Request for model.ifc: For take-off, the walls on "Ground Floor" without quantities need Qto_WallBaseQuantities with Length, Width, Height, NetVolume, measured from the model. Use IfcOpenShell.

First a look at what the model holds.

```python
import ifcopenshell
import ifcopenshell.util.element
import ifcopenshell.util.unit

model = ifcopenshell.open("model.ifc")
print(model.schema)
for unit_type in ("LENGTHUNIT", "AREAUNIT", "VOLUMEUNIT"):
    print(unit_type, ifcopenshell.util.unit.calculate_unit_scale(model, unit_type))
storey = next(s for s in model.by_type("IfcBuildingStorey") if s.Name == "Ground Floor")
walls = [e for e in ifcopenshell.util.element.get_decomposition(storey) if e.is_a("IfcWall")]
for e in sorted(walls, key=lambda e: e.id()):
    print(e.id(), e.is_a(), e.Name, list(ifcopenshell.util.element.get_psets(e, qtos_only=True)), sep=" | ")
```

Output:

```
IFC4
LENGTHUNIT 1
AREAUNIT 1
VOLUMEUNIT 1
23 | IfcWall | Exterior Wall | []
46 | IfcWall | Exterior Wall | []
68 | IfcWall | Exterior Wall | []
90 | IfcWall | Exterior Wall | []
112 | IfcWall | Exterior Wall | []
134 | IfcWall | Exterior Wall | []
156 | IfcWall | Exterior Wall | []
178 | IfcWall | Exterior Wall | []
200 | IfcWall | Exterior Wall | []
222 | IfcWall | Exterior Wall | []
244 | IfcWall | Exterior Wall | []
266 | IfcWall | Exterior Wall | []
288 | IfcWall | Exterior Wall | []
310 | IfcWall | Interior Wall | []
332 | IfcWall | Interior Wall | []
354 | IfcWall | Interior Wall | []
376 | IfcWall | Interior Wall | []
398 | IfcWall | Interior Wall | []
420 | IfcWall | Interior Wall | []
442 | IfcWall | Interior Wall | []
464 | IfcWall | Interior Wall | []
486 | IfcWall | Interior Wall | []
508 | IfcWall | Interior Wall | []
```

```python
import ifcopenshell
import ifcopenshell.api.pset
import ifcopenshell.geom
import ifcopenshell.util.element
import ifcopenshell.util.shape
import ifcopenshell.util.unit

model = ifcopenshell.open("model.ifc")
unit_scale = ifcopenshell.util.unit.calculate_unit_scale(model)
volume_scale = ifcopenshell.util.unit.calculate_unit_scale(model, "VOLUMEUNIT")
settings = ifcopenshell.geom.settings()

storey = next(s for s in model.by_type("IfcBuildingStorey") if s.Name == "Ground Floor")
walls = [e for e in ifcopenshell.util.element.get_decomposition(storey) if e.is_a("IfcWall")]

for e in sorted(walls, key=lambda e: e.id()):
    if ifcopenshell.util.element.get_psets(e, qtos_only=True, should_inherit=False):
        continue
    # Geometry comes back in metres, in the element's own axes.
    shape = ifcopenshell.geom.create_shape(settings, e)
    values = {
        "Length": ifcopenshell.util.shape.get_x(shape.geometry) / unit_scale,
        "Width": ifcopenshell.util.shape.get_y(shape.geometry) / unit_scale,
        "Height": ifcopenshell.util.shape.get_z(shape.geometry) / unit_scale,
        "NetVolume": ifcopenshell.util.shape.get_volume(shape.geometry) / volume_scale,
    }
    qto = ifcopenshell.api.pset.add_qto(model, product=e, name="Qto_WallBaseQuantities")
    ifcopenshell.api.pset.edit_qto(model, qto=qto, properties=values)
    print(e.id(), {k: round(v, 3) for k, v in values.items()})

model.write("model_v2.ifc")
```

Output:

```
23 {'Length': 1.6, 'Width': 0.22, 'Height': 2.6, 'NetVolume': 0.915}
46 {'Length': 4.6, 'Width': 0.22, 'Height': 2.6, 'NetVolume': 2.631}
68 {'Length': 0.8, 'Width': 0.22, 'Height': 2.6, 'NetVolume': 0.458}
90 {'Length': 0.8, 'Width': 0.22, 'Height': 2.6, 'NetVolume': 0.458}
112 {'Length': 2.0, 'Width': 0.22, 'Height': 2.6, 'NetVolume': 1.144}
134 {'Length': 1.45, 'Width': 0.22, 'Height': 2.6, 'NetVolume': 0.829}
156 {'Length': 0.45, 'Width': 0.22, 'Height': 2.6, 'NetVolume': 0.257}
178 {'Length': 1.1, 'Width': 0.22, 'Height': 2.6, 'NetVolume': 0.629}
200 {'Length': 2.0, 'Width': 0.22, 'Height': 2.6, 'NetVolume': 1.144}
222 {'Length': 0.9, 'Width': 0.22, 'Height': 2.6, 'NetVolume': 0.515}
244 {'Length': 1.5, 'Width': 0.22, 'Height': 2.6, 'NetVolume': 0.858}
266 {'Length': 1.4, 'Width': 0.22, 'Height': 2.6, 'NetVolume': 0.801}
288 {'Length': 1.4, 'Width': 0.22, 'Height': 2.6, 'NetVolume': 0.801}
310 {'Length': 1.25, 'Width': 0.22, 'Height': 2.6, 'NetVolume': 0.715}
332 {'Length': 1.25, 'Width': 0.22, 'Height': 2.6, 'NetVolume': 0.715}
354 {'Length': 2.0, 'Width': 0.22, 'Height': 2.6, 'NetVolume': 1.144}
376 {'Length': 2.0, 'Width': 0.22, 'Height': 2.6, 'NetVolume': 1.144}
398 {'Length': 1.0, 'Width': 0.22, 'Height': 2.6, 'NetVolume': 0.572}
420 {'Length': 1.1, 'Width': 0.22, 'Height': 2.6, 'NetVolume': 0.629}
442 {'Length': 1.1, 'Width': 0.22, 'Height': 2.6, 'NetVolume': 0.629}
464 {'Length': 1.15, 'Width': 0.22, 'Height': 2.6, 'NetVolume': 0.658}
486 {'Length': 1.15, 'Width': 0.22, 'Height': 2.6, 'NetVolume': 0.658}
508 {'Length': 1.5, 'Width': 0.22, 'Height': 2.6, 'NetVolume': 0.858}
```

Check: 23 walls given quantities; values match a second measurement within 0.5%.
